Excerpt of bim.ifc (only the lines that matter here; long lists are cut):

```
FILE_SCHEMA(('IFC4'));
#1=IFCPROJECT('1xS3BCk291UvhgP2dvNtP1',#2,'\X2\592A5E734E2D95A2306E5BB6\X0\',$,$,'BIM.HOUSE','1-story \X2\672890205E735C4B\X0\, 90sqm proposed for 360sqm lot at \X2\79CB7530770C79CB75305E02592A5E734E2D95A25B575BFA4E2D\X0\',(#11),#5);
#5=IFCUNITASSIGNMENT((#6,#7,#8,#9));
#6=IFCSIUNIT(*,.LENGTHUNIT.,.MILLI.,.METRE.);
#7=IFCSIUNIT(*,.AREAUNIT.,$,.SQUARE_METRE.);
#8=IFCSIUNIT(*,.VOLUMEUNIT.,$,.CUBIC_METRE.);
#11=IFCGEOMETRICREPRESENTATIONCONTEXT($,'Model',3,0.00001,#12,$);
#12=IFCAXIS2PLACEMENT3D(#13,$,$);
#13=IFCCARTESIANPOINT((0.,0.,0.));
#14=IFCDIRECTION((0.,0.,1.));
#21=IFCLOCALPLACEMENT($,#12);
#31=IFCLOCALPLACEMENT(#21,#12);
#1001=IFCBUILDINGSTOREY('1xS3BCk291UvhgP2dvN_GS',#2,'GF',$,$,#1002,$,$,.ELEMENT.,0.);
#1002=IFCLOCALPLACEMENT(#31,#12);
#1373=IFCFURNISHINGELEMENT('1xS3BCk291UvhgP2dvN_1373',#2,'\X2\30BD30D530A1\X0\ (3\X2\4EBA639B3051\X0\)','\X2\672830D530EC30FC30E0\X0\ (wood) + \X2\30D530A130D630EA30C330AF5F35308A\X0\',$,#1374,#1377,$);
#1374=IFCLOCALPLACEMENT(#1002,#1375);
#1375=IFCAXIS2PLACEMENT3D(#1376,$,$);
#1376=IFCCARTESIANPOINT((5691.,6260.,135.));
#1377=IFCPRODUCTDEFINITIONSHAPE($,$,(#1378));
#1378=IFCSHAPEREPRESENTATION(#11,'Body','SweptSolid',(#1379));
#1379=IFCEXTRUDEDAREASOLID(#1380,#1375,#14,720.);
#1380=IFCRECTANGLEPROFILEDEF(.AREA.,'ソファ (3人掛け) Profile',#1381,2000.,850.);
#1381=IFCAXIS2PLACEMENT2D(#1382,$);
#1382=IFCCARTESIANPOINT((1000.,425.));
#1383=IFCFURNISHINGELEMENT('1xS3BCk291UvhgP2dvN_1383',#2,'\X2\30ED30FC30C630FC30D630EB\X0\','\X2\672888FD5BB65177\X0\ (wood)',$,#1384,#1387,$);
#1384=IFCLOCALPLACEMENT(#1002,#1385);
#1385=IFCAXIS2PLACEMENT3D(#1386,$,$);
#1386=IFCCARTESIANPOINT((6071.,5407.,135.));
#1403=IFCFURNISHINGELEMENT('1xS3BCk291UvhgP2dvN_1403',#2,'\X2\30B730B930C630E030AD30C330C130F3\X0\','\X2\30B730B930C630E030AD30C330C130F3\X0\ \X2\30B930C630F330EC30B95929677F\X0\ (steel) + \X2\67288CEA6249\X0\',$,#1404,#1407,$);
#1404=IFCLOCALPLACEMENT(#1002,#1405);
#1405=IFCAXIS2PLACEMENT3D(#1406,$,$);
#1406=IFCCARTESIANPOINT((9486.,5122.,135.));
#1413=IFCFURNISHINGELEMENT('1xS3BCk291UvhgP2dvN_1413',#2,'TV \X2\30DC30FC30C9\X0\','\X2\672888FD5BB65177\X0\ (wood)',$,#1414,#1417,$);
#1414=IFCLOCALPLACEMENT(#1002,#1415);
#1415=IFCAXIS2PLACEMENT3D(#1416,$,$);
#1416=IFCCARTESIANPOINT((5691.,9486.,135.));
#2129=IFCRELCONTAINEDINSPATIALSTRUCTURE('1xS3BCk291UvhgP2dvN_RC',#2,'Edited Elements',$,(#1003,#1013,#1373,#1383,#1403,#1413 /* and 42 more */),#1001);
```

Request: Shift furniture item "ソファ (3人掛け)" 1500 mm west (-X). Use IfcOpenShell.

```python
import ifcopenshell
import ifcopenshell.api.geometry
import ifcopenshell.util.placement
import ifcopenshell.util.unit

model = ifcopenshell.open("bim.ifc")
unit_scale = ifcopenshell.util.unit.calculate_unit_scale(model)

item = model.by_guid("1xS3BCk291UvhgP2dvN_1373")
matrix = ifcopenshell.util.placement.get_local_placement(item.ObjectPlacement)
matrix[0, 3] -= 1.5 / unit_scale
ifcopenshell.api.geometry.edit_object_placement(model, product=item, matrix=matrix, is_si=False)

print(ifcopenshell.util.placement.get_local_placement(item.ObjectPlacement).round(3) + 0.0)

model.write("bim_rev.ifc")
```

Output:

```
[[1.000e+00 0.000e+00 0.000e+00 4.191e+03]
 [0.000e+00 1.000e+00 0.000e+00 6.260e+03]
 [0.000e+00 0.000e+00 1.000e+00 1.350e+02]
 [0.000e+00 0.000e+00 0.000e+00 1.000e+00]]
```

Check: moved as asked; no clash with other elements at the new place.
